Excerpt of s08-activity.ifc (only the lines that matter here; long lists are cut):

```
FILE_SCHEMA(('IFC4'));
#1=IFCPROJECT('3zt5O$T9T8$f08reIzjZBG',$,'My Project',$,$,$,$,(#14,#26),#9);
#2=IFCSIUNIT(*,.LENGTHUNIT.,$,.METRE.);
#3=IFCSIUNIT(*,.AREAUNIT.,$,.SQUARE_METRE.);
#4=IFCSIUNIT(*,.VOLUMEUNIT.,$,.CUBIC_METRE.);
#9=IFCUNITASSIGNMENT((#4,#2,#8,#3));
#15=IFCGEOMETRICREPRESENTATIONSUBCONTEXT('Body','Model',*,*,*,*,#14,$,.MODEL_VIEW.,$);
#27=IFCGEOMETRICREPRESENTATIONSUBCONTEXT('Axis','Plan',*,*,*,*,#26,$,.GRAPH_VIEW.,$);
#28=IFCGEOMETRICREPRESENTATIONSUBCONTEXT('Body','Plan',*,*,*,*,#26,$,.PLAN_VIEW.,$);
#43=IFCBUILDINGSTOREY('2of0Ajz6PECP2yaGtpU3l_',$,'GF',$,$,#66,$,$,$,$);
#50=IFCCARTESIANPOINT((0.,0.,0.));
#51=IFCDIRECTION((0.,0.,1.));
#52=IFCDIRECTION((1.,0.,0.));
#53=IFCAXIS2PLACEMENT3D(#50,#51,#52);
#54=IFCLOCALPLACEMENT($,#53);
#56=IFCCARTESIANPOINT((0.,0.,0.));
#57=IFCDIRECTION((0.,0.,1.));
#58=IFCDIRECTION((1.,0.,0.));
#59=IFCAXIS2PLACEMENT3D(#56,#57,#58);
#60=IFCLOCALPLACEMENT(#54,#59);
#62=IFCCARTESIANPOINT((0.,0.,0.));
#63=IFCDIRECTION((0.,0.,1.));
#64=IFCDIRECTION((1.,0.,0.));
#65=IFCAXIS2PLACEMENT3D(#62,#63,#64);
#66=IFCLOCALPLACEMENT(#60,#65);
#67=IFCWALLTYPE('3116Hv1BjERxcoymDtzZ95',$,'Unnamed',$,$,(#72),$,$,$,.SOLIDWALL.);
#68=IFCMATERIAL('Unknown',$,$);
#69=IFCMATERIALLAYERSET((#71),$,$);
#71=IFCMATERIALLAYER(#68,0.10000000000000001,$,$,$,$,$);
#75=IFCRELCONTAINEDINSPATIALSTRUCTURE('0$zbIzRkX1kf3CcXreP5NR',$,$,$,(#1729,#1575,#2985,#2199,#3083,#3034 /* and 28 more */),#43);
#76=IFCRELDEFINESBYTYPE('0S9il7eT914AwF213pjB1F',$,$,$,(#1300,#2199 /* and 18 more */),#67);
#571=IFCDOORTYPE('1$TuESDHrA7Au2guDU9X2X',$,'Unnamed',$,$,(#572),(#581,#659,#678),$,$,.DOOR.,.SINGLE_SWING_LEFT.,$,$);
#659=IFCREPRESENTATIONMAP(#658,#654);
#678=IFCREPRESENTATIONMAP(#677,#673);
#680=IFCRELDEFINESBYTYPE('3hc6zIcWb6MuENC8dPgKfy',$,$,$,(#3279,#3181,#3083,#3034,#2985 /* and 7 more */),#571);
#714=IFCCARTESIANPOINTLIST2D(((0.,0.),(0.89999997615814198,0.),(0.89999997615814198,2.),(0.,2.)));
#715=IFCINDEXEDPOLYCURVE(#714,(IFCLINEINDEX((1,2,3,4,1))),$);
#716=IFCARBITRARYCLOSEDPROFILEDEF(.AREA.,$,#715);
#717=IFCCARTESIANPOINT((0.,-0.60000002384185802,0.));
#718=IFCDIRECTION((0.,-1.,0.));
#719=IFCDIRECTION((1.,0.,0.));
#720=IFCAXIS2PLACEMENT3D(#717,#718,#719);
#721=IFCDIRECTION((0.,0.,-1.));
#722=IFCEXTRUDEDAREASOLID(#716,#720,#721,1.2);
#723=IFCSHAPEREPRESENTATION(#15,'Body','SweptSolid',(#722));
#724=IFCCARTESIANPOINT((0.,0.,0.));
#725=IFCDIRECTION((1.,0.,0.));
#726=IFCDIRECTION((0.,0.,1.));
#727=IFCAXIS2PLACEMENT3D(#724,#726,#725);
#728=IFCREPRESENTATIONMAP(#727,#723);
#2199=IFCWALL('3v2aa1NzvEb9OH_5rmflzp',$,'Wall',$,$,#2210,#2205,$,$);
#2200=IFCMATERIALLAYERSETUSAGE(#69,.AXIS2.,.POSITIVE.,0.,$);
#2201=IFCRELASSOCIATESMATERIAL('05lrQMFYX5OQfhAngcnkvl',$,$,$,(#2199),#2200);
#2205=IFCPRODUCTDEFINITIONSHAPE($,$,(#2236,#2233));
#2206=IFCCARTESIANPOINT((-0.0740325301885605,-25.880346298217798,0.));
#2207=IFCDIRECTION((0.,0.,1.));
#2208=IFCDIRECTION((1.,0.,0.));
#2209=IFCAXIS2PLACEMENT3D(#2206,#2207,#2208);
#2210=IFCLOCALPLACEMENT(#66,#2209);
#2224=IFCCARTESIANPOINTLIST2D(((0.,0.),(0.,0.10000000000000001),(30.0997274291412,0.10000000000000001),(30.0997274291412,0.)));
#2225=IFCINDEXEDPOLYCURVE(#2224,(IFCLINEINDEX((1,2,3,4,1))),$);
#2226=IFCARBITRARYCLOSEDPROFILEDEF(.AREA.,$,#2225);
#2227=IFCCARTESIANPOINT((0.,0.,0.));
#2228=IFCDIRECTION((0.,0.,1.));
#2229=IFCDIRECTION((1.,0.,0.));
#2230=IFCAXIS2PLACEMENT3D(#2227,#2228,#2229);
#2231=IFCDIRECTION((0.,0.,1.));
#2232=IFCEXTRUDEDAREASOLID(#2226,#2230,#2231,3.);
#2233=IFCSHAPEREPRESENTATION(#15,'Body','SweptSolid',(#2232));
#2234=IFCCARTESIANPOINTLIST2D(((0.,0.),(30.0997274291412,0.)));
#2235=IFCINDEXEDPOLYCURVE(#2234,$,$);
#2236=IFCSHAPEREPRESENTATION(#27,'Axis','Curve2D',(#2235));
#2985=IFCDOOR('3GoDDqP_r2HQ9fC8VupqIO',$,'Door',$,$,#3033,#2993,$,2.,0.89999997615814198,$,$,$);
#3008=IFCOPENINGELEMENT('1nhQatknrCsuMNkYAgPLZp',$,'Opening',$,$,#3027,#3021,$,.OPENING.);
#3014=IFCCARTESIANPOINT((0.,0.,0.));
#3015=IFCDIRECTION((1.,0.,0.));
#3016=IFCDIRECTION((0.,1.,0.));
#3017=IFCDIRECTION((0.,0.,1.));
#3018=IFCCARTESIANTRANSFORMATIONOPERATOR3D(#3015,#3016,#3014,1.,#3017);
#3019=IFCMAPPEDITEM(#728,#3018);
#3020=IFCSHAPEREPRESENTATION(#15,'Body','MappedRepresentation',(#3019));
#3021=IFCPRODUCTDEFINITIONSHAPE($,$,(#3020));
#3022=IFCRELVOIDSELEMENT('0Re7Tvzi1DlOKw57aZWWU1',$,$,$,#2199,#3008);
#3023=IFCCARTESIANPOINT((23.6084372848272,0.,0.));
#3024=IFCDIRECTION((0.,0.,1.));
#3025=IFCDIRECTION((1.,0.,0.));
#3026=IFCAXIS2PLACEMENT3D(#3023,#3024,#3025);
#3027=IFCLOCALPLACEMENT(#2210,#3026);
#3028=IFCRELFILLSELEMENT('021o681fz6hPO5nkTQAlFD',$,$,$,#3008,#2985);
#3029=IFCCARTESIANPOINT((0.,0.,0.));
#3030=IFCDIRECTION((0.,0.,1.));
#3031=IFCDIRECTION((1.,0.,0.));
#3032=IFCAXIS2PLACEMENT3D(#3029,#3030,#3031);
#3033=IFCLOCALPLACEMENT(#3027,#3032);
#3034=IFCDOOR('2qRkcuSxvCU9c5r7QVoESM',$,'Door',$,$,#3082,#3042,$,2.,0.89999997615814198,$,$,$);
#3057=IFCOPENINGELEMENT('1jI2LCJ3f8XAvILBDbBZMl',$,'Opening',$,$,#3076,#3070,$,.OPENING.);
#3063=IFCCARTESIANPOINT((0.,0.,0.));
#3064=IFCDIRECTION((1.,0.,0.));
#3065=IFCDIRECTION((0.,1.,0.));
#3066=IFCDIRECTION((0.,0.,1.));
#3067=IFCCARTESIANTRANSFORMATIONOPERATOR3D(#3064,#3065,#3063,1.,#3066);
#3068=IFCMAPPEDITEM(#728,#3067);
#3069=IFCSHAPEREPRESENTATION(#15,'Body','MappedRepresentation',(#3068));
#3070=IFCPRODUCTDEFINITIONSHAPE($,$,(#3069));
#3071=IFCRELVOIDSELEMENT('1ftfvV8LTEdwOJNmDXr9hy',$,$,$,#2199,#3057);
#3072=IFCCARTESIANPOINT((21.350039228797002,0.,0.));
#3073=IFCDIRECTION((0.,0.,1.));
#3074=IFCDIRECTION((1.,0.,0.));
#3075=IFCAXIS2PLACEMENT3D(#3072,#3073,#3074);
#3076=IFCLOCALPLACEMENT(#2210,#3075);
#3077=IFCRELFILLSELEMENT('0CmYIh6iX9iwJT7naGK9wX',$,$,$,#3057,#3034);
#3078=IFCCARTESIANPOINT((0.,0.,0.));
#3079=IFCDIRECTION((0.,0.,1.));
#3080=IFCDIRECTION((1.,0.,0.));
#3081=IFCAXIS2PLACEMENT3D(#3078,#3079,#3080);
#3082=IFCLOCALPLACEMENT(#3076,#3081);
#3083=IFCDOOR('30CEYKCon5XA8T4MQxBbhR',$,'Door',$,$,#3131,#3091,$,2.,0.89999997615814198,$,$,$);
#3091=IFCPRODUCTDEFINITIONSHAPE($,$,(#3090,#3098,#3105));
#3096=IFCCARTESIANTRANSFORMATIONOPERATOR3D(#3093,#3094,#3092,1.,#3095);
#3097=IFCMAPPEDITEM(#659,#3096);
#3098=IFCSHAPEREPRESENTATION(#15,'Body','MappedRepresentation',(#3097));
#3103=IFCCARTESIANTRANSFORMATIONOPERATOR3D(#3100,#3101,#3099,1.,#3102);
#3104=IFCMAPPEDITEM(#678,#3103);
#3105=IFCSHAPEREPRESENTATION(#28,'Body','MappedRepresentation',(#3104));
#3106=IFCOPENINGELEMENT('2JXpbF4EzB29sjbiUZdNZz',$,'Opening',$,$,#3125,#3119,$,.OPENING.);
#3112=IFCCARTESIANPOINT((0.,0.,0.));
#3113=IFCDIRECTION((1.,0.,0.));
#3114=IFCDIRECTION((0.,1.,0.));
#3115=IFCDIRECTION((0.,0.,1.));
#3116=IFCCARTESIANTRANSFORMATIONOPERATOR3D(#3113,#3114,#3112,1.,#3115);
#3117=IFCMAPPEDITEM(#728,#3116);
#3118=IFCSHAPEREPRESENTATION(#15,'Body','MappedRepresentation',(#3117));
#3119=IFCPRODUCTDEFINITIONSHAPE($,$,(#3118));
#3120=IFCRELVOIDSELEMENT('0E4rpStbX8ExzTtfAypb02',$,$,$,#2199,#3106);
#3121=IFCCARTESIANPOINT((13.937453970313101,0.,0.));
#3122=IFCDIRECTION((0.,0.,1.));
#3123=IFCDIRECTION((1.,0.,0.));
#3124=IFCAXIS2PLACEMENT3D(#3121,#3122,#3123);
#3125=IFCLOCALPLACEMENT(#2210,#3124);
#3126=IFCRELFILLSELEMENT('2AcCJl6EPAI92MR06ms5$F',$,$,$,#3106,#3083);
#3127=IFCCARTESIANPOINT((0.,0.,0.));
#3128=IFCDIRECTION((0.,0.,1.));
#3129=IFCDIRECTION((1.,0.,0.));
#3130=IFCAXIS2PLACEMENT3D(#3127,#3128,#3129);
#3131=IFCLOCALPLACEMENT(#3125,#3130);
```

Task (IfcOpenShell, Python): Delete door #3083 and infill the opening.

```python
import ifcopenshell
import ifcopenshell.api.feature
import ifcopenshell.api.root
import ifcopenshell.geom
import ifcopenshell.util.shape

model = ifcopenshell.open("s08-activity.ifc")
settings = ifcopenshell.geom.settings()


def volume(element):
    """Net volume in cubic metres, openings subtracted."""
    shape = ifcopenshell.geom.create_shape(settings, element)
    return ifcopenshell.util.shape.get_volume(shape.geometry)


door = model.by_id(3083)
opening = door.FillsVoids[0].RelatingOpeningElement
wall = opening.VoidsElements[0].RelatingBuildingElement
before = volume(wall)

ifcopenshell.api.root.remove_product(model, product=door)
ifcopenshell.api.feature.remove_feature(model, feature=opening)

after = volume(wall)

print(f"wall volume {before:.3f} -> {after:.3f} m3")

model.write("s08-activity_rev.ifc")
```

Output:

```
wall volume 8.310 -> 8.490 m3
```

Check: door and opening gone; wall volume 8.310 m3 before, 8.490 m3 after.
